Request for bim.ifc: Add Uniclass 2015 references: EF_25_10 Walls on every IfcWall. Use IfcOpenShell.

First a look at what the model holds.

```python
import ifcopenshell

model = ifcopenshell.open("bim.ifc")
print(model.schema)
print("classifications:", [c.Name for c in model.by_type("IfcClassification")])
for ifc_class in ("IfcDoor", "IfcRoof", "IfcStair", "IfcWall", "IfcWindow"):
    print(ifc_class, len(model.by_type(ifc_class)))
```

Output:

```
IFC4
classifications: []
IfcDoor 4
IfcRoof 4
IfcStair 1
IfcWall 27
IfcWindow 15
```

```python
import ifcopenshell
import ifcopenshell.api.classification

model = ifcopenshell.open("bim.ifc")

system = ifcopenshell.api.classification.add_classification(model, classification="Uniclass 2015")

codes = {
    "IfcWall": ("EF_25_10", "Walls"),
}
for ifc_class, (code, name) in codes.items():
    products = model.by_type(ifc_class)
    ifcopenshell.api.classification.add_reference(
        model, products=products, classification=system, identification=code, name=name
    )
    print(code, len(products))

model.write("bim_rev.ifc")
```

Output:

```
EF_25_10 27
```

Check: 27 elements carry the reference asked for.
